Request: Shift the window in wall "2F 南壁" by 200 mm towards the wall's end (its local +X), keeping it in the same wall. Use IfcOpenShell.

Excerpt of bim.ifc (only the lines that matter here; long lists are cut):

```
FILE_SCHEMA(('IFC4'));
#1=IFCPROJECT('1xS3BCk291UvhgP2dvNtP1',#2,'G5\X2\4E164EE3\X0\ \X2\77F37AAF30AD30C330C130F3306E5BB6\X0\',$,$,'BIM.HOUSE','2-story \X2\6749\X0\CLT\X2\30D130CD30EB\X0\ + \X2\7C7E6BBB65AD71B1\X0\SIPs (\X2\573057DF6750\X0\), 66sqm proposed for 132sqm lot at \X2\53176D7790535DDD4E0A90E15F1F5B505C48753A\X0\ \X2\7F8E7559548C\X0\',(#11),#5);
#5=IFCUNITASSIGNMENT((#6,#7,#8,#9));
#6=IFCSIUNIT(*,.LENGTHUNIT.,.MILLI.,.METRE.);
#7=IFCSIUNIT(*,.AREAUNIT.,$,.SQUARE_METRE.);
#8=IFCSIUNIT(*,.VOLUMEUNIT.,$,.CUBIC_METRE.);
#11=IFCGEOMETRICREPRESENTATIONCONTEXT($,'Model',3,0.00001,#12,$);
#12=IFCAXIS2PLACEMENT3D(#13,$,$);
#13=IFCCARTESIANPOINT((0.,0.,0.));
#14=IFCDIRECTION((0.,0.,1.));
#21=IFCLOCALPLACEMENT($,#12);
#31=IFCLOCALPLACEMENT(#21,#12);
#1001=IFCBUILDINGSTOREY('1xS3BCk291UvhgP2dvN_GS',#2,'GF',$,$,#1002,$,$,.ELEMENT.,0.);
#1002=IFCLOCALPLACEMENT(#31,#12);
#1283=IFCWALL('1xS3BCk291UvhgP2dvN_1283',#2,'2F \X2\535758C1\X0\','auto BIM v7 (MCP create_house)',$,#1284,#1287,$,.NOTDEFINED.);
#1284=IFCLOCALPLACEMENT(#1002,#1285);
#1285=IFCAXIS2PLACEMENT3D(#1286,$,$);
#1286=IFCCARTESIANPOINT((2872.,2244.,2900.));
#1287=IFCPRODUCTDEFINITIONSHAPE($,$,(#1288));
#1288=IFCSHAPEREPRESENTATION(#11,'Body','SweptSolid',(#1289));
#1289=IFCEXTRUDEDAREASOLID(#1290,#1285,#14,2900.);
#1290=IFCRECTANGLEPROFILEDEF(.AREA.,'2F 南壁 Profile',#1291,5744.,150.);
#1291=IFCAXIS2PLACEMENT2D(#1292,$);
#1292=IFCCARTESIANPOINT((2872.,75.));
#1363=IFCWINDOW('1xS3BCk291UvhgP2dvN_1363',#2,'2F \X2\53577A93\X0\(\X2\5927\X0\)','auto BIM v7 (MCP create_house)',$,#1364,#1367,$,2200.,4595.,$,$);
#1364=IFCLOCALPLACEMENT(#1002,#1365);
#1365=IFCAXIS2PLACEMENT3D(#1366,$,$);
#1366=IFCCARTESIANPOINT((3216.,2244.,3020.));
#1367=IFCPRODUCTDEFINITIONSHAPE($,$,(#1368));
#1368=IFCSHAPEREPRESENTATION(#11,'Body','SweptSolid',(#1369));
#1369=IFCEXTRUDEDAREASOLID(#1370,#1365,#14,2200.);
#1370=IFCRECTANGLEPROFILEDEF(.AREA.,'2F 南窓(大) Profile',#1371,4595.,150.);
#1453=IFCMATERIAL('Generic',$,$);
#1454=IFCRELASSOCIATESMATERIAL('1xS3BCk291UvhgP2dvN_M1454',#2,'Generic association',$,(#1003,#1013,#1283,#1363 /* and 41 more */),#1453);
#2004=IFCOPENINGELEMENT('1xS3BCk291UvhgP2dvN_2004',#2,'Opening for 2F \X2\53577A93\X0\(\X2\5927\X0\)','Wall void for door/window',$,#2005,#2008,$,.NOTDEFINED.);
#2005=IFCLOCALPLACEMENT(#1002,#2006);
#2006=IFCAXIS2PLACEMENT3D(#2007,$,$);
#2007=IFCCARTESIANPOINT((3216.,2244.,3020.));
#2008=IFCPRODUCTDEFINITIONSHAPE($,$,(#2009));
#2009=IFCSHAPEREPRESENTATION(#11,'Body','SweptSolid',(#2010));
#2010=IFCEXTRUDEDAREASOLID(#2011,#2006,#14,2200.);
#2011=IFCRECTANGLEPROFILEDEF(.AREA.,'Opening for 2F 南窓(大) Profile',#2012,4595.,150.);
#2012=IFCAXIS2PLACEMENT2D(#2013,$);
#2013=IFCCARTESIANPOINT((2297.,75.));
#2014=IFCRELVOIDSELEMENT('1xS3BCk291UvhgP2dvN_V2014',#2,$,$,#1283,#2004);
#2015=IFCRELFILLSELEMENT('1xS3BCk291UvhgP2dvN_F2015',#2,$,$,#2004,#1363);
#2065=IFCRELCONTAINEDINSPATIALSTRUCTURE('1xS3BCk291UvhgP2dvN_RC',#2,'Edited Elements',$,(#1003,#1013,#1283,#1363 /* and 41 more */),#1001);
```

```python
import ifcopenshell
import ifcopenshell.api.geometry
import ifcopenshell.util.placement
import ifcopenshell.util.unit

model = ifcopenshell.open("bim.ifc")
unit_scale = ifcopenshell.util.unit.calculate_unit_scale(model)

window = model.by_guid("1xS3BCk291UvhgP2dvN_1363")
opening = window.FillsVoids[0].RelatingOpeningElement
wall = opening.VoidsElements[0].RelatingBuildingElement

wall_matrix = ifcopenshell.util.placement.get_local_placement(wall.ObjectPlacement)
shift = wall_matrix[:3, 0] * 0.2 / unit_scale
before = ifcopenshell.util.placement.get_local_placement(window.ObjectPlacement)[:3, 3].copy()

# The window is not placed relative to its opening, so move both.
for product in (opening, window):
    matrix = ifcopenshell.util.placement.get_local_placement(product.ObjectPlacement)
    matrix[:3, 3] += shift
    ifcopenshell.api.geometry.edit_object_placement(model, product=product, matrix=matrix, is_si=False)

after = ifcopenshell.util.placement.get_local_placement(window.ObjectPlacement)[:3, 3]
print("window moved by", (after - before).round(3) + 0.0)

model.write("bim-out.ifc")
```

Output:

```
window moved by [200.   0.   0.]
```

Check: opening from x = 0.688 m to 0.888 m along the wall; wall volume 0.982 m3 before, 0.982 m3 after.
